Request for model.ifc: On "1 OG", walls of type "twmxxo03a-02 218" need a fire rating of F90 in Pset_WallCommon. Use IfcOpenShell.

First a look at what the model holds.

```python
import ifcopenshell
import ifcopenshell.util.element

model = ifcopenshell.open("model.ifc")
print(model.schema)
storey = next(s for s in model.by_type("IfcBuildingStorey") if s.Name == "1 OG")
walls = [e for e in ifcopenshell.util.element.get_decomposition(storey) if e.is_a("IfcWall")]
seen = {}
for e in walls:
    element_type = ifcopenshell.util.element.get_type(e)
    key = (element_type.Name if element_type != e and element_type else None, ifcopenshell.util.element.get_pset(e, "Pset_WallCommon", "FireRating"))
    seen[key] = seen.get(key, 0) + 1
for (name, value), count in sorted(seen.items(), key=str):
    print(count, "x", name, "|", value)
```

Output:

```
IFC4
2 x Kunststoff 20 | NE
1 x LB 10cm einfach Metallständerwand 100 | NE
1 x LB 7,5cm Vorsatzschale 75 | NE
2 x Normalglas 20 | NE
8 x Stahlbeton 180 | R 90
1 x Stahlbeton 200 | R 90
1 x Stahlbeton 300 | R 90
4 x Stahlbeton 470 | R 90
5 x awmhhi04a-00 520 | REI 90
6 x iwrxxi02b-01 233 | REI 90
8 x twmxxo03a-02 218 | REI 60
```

```python
import ifcopenshell
import ifcopenshell.api.pset
import ifcopenshell.util.element

model = ifcopenshell.open("model.ifc")

storey = next(s for s in model.by_type("IfcBuildingStorey") if s.Name == "1 OG")
walls = [e for e in ifcopenshell.util.element.get_decomposition(storey) if e.is_a("IfcWall")]

count = 0
for e in walls:
    element_type = ifcopenshell.util.element.get_type(e)
    if element_type in (None, e) or element_type.Name != "twmxxo03a-02 218":
        continue
    # add_pset returns the element's existing set when there is one.
    pset = ifcopenshell.api.pset.add_pset(model, product=e, name="Pset_WallCommon")
    ifcopenshell.api.pset.edit_pset(model, pset=pset, properties={"FireRating": "F90"})
    count += 1

print(count, "walls updated")

model.write("model_v2.ifc")
```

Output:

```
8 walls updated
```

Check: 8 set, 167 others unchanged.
